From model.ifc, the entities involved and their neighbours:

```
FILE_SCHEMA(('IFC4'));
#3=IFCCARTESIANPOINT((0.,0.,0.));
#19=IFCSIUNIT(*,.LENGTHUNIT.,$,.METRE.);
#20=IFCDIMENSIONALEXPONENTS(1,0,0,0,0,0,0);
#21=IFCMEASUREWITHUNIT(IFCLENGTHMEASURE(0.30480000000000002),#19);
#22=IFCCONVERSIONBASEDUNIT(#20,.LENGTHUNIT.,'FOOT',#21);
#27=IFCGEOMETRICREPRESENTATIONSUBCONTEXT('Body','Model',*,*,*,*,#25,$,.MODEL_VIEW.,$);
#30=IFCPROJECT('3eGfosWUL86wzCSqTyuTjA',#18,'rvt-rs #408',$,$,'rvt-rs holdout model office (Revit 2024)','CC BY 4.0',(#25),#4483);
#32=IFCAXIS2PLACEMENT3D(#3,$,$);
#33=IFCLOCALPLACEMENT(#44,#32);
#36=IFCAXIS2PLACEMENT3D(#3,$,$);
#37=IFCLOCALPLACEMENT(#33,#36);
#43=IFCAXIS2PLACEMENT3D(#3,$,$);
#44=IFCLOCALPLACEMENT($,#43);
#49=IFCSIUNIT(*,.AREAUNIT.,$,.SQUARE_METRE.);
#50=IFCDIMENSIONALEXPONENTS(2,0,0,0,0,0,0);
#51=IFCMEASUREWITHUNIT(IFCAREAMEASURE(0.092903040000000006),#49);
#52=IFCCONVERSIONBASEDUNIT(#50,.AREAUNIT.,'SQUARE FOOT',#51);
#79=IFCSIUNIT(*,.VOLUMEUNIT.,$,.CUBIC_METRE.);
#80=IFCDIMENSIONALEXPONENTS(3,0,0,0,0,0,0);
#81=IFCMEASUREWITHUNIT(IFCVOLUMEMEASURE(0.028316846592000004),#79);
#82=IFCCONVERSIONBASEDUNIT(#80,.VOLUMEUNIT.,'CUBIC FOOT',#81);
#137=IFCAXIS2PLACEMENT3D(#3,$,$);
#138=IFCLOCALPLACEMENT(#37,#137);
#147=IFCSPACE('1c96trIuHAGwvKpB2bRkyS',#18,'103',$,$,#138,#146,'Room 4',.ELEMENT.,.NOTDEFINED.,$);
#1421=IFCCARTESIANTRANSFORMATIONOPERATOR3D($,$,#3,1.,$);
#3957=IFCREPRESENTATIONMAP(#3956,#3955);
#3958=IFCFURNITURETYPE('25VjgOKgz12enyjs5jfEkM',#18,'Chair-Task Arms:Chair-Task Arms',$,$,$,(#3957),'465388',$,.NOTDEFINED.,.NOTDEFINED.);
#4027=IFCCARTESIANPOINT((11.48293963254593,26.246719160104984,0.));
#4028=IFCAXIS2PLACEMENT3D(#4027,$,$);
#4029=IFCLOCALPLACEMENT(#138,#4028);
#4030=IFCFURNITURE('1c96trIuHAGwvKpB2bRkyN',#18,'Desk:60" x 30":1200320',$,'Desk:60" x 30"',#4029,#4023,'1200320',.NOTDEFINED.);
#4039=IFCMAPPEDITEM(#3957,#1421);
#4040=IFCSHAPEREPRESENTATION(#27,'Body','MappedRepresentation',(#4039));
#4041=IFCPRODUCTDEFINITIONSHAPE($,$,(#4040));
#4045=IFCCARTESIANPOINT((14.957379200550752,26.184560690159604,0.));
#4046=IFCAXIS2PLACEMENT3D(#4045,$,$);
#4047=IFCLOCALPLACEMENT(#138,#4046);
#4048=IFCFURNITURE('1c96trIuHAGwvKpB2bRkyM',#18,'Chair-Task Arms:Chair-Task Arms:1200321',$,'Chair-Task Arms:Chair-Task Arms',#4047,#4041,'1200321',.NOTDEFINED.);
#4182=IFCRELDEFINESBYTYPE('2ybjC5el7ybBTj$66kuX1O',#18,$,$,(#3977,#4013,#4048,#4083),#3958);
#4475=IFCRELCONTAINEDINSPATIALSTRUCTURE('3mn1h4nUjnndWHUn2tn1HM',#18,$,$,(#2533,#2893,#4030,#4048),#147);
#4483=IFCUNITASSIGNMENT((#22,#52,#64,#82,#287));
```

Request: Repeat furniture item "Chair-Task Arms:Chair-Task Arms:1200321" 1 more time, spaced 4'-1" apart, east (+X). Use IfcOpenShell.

```python
import numpy as np
import ifcopenshell
import ifcopenshell.api.geometry
import ifcopenshell.api.root
import ifcopenshell.util.element
import ifcopenshell.util.placement
import ifcopenshell.util.unit

model = ifcopenshell.open("model.ifc")
unit_scale = ifcopenshell.util.unit.calculate_unit_scale(model)


def reuse_history(source, copy):
    """copy_class also copies each property set's owner history, people and application; keep the originals."""
    for rel in copy.IsDefinedBy:
        if rel.is_a("IfcRelDefinesByProperties") and (history := rel.RelatingPropertyDefinition.OwnerHistory):
            rel.RelatingPropertyDefinition.OwnerHistory = source.OwnerHistory
            ifcopenshell.util.element.remove_deep2(model, history)


source = model.by_id(4048)
base = ifcopenshell.util.placement.get_local_placement(source.ObjectPlacement)
step = np.array([1.0, 0.0, 0.0]) * 49 * 0.0254 / unit_scale

for i in range(1, 2):
    copy = ifcopenshell.api.root.copy_class(model, product=source)
    copy.Representation = ifcopenshell.util.element.copy_deep(
        model, source.Representation, exclude=["IfcGeometricRepresentationContext", "IfcRepresentationMap"]
    )
    copy.Name = "Chair-Task Arms:Chair-Task Arms"
    copy.Tag = None
    reuse_history(source, copy)
    matrix = base.copy()
    matrix[:3, 3] += i * step
    print("added at", matrix[:3, 3].round(3) + 0.0)
    ifcopenshell.api.geometry.edit_object_placement(model, product=copy, matrix=matrix, is_si=False)

model.write("model_v2.ifc")
```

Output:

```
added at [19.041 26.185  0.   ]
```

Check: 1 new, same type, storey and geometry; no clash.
